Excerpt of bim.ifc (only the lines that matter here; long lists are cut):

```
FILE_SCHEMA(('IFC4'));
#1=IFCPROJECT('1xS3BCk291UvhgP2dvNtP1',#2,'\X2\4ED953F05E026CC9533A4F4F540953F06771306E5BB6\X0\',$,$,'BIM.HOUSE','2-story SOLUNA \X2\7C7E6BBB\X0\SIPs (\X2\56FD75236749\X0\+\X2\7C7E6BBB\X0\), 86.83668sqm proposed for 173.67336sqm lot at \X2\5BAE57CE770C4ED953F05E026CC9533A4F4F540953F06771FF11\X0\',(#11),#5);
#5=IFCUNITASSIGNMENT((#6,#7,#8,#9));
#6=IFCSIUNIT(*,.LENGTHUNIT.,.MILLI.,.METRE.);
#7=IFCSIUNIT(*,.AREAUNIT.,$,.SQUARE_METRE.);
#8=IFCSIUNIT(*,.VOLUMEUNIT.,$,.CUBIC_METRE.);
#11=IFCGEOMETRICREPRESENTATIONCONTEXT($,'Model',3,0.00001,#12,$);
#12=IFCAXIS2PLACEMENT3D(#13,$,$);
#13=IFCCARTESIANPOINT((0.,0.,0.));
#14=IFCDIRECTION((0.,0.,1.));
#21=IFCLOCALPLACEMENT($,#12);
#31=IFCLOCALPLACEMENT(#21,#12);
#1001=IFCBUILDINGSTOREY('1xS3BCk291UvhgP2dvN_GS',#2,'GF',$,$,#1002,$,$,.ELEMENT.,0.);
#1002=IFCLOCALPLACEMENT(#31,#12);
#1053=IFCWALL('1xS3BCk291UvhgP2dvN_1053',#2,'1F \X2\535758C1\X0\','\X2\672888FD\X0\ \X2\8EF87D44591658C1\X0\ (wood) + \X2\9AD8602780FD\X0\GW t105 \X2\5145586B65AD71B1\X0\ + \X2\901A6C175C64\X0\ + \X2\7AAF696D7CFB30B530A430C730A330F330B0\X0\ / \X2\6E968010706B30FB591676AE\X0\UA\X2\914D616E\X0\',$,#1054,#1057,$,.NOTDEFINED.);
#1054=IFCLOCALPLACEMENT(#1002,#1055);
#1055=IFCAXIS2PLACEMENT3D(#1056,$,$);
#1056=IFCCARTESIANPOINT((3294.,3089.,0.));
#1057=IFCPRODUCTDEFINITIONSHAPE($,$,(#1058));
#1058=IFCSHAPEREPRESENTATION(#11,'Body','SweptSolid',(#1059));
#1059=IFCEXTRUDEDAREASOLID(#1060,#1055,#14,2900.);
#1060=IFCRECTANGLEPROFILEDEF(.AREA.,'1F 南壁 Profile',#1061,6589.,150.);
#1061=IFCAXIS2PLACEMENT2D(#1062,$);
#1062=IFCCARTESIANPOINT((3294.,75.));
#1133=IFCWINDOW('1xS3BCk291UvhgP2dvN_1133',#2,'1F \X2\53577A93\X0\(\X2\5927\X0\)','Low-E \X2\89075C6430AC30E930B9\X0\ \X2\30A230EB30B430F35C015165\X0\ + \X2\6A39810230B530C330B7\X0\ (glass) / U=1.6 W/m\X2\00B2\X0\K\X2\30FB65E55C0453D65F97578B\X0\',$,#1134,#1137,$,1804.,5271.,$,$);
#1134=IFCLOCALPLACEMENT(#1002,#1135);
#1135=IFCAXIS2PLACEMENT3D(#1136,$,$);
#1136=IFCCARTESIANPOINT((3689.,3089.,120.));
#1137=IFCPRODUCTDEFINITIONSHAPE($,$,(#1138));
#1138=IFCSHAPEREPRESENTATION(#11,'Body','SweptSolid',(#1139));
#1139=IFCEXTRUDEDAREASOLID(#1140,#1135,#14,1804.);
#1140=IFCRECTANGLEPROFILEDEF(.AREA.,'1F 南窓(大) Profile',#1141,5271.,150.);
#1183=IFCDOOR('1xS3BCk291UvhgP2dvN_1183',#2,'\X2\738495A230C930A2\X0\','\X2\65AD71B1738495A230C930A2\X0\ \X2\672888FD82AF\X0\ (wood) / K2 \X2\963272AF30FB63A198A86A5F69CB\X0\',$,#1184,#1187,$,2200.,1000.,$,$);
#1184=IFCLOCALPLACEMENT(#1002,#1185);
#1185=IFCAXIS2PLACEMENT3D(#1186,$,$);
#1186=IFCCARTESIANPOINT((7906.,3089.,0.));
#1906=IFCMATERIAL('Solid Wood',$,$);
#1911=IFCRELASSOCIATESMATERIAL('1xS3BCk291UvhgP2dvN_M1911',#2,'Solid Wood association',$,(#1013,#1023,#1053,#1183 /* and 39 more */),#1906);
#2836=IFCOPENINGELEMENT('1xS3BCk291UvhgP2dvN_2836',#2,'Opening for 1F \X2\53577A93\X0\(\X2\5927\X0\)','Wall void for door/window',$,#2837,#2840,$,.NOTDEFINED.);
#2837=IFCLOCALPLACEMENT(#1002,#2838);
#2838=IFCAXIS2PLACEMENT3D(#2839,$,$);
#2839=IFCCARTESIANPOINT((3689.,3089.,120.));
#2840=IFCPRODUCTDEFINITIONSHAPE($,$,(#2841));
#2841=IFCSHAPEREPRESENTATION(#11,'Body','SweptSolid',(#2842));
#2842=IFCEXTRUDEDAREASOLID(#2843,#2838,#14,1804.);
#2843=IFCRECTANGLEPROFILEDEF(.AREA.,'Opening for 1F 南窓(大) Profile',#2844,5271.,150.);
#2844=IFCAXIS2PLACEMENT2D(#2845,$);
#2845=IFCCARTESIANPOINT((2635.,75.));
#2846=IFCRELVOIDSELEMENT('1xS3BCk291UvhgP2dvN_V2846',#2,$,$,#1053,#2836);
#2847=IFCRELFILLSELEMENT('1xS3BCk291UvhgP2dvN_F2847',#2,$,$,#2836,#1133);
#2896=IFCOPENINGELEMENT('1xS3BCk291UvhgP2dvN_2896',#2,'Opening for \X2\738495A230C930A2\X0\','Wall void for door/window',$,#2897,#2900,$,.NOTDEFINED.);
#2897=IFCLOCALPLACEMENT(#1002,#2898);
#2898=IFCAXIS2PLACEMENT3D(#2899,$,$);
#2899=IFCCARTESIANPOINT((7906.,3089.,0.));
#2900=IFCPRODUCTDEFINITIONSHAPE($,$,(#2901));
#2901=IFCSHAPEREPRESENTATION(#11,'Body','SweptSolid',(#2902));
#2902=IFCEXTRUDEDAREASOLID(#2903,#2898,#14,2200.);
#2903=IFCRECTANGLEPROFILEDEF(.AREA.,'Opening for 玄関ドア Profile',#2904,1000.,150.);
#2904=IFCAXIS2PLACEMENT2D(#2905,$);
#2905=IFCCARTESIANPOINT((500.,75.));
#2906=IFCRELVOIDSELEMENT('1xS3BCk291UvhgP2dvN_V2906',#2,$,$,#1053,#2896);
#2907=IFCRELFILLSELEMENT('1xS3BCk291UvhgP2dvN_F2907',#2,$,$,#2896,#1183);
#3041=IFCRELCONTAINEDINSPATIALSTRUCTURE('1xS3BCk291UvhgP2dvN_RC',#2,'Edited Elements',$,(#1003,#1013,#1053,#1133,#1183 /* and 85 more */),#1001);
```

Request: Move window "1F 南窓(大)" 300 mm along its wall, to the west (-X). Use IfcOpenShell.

```python
import ifcopenshell
import ifcopenshell.api.geometry
import ifcopenshell.util.placement
import ifcopenshell.util.unit

model = ifcopenshell.open("bim.ifc")
unit_scale = ifcopenshell.util.unit.calculate_unit_scale(model)

window = model.by_guid("1xS3BCk291UvhgP2dvN_1133")
opening = window.FillsVoids[0].RelatingOpeningElement
wall = opening.VoidsElements[0].RelatingBuildingElement

wall_matrix = ifcopenshell.util.placement.get_local_placement(wall.ObjectPlacement)
shift = wall_matrix[:3, 0] * -0.3 / unit_scale
before = ifcopenshell.util.placement.get_local_placement(window.ObjectPlacement)[:3, 3].copy()

# The window is not placed relative to its opening, so move both.
for product in (opening, window):
    matrix = ifcopenshell.util.placement.get_local_placement(product.ObjectPlacement)
    matrix[:3, 3] += shift
    ifcopenshell.api.geometry.edit_object_placement(model, product=product, matrix=matrix, is_si=False)

after = ifcopenshell.util.placement.get_local_placement(window.ObjectPlacement)[:3, 3]
print("window moved by", (after - before).round(3) + 0.0)

model.write("bim-out.ifc")
```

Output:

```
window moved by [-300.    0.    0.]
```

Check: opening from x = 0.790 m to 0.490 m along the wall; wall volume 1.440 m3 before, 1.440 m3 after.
